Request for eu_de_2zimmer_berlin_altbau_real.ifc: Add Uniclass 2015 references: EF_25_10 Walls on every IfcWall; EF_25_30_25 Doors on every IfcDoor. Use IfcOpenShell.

First a look at what the model holds.

```python
import ifcopenshell

model = ifcopenshell.open("eu_de_2zimmer_berlin_altbau_real.ifc")
print(model.schema)
print("classifications:", [c.Name for c in model.by_type("IfcClassification")])
for ifc_class in ("IfcDoor", "IfcRoof", "IfcStair", "IfcWall", "IfcWindow"):
    print(ifc_class, len(model.by_type(ifc_class)))
```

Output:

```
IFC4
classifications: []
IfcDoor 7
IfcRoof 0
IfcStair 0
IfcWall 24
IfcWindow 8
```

```python
import ifcopenshell
import ifcopenshell.api.classification

model = ifcopenshell.open("eu_de_2zimmer_berlin_altbau_real.ifc")

system = ifcopenshell.api.classification.add_classification(model, classification="Uniclass 2015")

codes = {
    "IfcWall": ("EF_25_10", "Walls"),
    "IfcDoor": ("EF_25_30_25", "Doors"),
}
for ifc_class, (code, name) in codes.items():
    products = model.by_type(ifc_class)
    ifcopenshell.api.classification.add_reference(
        model, products=products, classification=system, identification=code, name=name
    )
    print(code, len(products))

model.write("eu_de_2zimmer_berlin_altbau_real-out.ifc")
```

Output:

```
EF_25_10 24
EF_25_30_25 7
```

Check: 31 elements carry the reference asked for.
